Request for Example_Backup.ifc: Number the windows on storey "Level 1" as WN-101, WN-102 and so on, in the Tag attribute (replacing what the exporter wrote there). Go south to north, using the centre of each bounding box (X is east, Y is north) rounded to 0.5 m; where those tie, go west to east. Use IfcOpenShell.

First a look at what the model holds.

```python
import ifcopenshell
import ifcopenshell.util.element
import ifcopenshell.util.placement

model = ifcopenshell.open("Example_Backup.ifc")
print(model.schema)
storey = next(s for s in model.by_type("IfcBuildingStorey") if s.Name == "Level 1")
windows = [e for e in ifcopenshell.util.element.get_decomposition(storey) if e.is_a("IfcWindow")]
for e in sorted(windows, key=lambda e: e.id()):
    origin = ifcopenshell.util.placement.get_local_placement(e.ObjectPlacement)[:3, 3]
    print(e.id(), e.Tag, e.Name, origin.round(2) + 0.0, sep=" | ")
```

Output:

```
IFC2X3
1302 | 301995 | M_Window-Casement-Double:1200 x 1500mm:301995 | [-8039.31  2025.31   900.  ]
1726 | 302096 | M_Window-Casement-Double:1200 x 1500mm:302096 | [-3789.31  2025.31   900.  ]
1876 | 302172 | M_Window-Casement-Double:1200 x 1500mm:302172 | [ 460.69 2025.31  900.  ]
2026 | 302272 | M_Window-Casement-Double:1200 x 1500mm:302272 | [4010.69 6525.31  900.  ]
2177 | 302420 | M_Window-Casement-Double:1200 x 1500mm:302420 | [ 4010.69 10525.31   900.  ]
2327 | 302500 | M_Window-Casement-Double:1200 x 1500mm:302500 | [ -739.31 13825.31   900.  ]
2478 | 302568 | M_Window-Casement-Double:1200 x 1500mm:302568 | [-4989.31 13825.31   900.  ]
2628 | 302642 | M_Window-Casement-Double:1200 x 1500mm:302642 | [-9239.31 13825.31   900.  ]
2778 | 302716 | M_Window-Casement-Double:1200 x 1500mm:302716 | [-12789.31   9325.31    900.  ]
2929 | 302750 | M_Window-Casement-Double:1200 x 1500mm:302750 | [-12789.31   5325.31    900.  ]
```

```python
import ifcopenshell
import ifcopenshell.geom
import ifcopenshell.util.element
import ifcopenshell.util.shape

model = ifcopenshell.open("Example_Backup.ifc")
settings = ifcopenshell.geom.settings()
settings.set("use-world-coords", True)


def centre(element):
    shape = ifcopenshell.geom.create_shape(settings, element)
    return ifcopenshell.util.shape.get_bbox_centroid(shape.geometry)


storey = next(s for s in model.by_type("IfcBuildingStorey") if s.Name == "Level 1")
windows = [e for e in ifcopenshell.util.element.get_decomposition(storey) if e.is_a("IfcWindow")]

# Insertion points can sit at a corner or the storey origin, so sort by the geometry (in metres).
centres = {e: centre(e) for e in windows}
windows.sort(key=lambda e: (round(centres[e][1] / 0.5), centres[e][0]))

for i, e in enumerate(windows, start=1):
    number = f"WN-1{i:02d}"
    e.Tag = number
    print(e.id(), number)

model.write("Example_Backup_updated.ifc")
```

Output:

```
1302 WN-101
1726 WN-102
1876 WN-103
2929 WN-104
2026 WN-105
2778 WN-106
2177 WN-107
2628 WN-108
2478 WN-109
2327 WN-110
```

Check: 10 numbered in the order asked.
